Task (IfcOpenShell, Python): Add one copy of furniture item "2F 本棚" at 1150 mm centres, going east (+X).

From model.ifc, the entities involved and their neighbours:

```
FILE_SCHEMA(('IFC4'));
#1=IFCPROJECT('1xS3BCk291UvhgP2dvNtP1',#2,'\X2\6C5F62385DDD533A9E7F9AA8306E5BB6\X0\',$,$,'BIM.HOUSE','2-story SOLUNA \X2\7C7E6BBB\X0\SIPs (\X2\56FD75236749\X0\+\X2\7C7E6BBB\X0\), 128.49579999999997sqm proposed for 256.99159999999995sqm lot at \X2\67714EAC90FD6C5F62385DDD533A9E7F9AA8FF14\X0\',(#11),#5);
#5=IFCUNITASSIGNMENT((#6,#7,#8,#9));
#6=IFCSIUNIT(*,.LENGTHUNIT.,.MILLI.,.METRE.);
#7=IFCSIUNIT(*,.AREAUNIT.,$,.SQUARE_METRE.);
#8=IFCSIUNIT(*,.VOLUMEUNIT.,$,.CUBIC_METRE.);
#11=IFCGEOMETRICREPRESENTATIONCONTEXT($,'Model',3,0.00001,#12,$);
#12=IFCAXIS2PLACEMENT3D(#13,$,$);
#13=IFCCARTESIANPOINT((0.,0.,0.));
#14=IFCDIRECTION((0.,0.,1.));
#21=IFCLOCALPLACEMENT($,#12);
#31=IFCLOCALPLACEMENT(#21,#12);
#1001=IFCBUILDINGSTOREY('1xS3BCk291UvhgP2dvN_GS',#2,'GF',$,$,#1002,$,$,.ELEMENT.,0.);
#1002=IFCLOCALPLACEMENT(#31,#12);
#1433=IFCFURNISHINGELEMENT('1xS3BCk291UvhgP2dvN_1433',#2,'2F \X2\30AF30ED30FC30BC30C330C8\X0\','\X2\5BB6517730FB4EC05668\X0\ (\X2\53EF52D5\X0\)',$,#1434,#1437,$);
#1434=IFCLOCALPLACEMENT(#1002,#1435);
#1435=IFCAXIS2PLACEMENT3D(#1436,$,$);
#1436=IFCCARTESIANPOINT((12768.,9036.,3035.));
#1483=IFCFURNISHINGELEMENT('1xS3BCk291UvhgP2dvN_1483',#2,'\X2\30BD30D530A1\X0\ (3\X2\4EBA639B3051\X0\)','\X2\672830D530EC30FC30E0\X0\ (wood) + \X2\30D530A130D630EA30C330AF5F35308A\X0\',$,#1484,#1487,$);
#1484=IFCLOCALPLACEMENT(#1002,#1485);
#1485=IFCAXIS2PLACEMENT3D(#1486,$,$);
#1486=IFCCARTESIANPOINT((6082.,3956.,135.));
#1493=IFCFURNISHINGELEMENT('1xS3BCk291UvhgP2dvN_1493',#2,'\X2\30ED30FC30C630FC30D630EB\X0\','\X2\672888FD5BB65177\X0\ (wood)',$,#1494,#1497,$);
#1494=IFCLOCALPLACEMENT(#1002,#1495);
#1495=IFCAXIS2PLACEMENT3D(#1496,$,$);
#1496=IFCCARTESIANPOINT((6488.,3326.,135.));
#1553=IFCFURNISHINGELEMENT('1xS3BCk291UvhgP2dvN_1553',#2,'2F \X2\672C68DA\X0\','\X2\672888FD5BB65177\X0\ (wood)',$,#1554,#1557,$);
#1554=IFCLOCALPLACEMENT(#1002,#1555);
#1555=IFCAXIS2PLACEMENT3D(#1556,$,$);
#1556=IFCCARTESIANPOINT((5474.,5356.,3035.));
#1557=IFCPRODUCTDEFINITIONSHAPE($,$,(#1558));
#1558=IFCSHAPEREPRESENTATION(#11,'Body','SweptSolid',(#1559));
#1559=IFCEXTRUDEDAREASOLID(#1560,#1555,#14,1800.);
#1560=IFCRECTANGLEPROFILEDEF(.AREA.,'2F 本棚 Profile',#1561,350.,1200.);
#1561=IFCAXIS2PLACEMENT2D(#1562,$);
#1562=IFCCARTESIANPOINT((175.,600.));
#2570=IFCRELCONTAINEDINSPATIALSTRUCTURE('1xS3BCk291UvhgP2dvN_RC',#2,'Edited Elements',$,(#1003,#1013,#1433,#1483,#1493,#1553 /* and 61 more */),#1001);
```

```python
import numpy as np
import ifcopenshell
import ifcopenshell.api.geometry
import ifcopenshell.api.root
import ifcopenshell.util.element
import ifcopenshell.util.placement
import ifcopenshell.util.unit

model = ifcopenshell.open("model.ifc")
unit_scale = ifcopenshell.util.unit.calculate_unit_scale(model)


def reuse_history(source, copy):
    """copy_class also copies each property set's owner history, people and application; keep the originals."""
    for rel in copy.IsDefinedBy:
        if rel.is_a("IfcRelDefinesByProperties") and (history := rel.RelatingPropertyDefinition.OwnerHistory):
            rel.RelatingPropertyDefinition.OwnerHistory = source.OwnerHistory
            ifcopenshell.util.element.remove_deep2(model, history)


source = model.by_id(1553)
base = ifcopenshell.util.placement.get_local_placement(source.ObjectPlacement)
step = np.array([1.0, 0.0, 0.0]) * 1.15 / unit_scale

for i in range(1, 2):
    copy = ifcopenshell.api.root.copy_class(model, product=source)
    copy.Representation = ifcopenshell.util.element.copy_deep(
        model, source.Representation, exclude=["IfcGeometricRepresentationContext", "IfcRepresentationMap"]
    )
    reuse_history(source, copy)
    matrix = base.copy()
    matrix[:3, 3] += i * step
    print("added at", matrix[:3, 3].round(3) + 0.0)
    ifcopenshell.api.geometry.edit_object_placement(model, product=copy, matrix=matrix, is_si=False)

model.write("model_updated.ifc")
```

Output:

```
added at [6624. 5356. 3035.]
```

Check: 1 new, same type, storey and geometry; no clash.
